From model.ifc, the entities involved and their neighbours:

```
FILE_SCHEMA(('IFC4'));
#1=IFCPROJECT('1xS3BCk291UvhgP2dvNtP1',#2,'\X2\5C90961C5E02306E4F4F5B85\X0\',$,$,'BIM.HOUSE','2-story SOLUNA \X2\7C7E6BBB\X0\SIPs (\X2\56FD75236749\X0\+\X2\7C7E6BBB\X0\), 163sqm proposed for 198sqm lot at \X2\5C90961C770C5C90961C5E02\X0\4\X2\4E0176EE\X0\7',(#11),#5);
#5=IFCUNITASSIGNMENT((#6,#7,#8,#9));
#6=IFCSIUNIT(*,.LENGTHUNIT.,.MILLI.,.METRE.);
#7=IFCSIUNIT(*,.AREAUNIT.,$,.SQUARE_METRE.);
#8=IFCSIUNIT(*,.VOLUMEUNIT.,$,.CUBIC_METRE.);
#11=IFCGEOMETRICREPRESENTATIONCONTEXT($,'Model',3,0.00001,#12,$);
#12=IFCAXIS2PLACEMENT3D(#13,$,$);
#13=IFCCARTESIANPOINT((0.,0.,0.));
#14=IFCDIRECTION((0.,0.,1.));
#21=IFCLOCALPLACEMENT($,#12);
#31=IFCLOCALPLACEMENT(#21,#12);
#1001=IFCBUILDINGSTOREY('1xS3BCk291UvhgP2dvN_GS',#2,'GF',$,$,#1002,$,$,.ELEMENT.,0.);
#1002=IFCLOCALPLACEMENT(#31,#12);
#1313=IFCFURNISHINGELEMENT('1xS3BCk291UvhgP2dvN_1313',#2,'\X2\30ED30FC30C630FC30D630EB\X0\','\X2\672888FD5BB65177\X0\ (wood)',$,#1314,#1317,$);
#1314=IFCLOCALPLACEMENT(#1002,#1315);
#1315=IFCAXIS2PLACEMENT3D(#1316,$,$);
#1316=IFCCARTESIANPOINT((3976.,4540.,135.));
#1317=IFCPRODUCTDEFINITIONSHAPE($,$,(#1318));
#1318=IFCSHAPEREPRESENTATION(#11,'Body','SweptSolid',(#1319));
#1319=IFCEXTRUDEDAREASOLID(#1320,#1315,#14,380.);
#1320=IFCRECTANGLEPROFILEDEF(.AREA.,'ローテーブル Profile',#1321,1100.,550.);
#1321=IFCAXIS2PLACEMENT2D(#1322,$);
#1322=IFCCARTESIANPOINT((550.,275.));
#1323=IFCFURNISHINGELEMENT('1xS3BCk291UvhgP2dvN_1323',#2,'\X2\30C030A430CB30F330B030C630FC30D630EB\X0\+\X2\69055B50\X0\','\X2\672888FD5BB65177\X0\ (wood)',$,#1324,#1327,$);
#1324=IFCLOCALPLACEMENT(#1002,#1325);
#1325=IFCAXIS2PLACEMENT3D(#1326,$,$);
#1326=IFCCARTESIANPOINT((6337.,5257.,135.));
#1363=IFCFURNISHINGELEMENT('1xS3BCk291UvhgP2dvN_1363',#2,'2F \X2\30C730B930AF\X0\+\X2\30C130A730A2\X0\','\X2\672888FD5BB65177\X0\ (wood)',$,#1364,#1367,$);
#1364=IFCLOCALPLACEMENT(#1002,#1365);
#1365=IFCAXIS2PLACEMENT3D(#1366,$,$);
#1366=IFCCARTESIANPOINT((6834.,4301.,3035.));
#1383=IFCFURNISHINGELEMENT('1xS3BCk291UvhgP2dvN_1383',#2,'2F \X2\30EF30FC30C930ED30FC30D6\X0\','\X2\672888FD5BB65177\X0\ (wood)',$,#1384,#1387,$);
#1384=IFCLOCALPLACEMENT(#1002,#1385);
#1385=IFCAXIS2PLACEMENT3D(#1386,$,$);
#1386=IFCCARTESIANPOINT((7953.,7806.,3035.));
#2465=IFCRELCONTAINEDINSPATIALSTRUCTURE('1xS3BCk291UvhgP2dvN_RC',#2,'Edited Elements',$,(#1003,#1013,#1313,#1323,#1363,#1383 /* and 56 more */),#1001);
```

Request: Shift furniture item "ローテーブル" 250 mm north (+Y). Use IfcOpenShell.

```python
import ifcopenshell
import ifcopenshell.api.geometry
import ifcopenshell.util.placement
import ifcopenshell.util.unit

model = ifcopenshell.open("model.ifc")
unit_scale = ifcopenshell.util.unit.calculate_unit_scale(model)

item = model.by_id(1313)
matrix = ifcopenshell.util.placement.get_local_placement(item.ObjectPlacement)
matrix[1, 3] += 0.25 / unit_scale
ifcopenshell.api.geometry.edit_object_placement(model, product=item, matrix=matrix, is_si=False)

print(ifcopenshell.util.placement.get_local_placement(item.ObjectPlacement).round(3) + 0.0)

model.write("model-out.ifc")
```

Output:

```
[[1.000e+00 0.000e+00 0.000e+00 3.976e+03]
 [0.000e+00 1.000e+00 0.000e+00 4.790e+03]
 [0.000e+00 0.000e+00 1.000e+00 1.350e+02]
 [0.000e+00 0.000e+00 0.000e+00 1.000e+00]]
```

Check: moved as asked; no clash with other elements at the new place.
